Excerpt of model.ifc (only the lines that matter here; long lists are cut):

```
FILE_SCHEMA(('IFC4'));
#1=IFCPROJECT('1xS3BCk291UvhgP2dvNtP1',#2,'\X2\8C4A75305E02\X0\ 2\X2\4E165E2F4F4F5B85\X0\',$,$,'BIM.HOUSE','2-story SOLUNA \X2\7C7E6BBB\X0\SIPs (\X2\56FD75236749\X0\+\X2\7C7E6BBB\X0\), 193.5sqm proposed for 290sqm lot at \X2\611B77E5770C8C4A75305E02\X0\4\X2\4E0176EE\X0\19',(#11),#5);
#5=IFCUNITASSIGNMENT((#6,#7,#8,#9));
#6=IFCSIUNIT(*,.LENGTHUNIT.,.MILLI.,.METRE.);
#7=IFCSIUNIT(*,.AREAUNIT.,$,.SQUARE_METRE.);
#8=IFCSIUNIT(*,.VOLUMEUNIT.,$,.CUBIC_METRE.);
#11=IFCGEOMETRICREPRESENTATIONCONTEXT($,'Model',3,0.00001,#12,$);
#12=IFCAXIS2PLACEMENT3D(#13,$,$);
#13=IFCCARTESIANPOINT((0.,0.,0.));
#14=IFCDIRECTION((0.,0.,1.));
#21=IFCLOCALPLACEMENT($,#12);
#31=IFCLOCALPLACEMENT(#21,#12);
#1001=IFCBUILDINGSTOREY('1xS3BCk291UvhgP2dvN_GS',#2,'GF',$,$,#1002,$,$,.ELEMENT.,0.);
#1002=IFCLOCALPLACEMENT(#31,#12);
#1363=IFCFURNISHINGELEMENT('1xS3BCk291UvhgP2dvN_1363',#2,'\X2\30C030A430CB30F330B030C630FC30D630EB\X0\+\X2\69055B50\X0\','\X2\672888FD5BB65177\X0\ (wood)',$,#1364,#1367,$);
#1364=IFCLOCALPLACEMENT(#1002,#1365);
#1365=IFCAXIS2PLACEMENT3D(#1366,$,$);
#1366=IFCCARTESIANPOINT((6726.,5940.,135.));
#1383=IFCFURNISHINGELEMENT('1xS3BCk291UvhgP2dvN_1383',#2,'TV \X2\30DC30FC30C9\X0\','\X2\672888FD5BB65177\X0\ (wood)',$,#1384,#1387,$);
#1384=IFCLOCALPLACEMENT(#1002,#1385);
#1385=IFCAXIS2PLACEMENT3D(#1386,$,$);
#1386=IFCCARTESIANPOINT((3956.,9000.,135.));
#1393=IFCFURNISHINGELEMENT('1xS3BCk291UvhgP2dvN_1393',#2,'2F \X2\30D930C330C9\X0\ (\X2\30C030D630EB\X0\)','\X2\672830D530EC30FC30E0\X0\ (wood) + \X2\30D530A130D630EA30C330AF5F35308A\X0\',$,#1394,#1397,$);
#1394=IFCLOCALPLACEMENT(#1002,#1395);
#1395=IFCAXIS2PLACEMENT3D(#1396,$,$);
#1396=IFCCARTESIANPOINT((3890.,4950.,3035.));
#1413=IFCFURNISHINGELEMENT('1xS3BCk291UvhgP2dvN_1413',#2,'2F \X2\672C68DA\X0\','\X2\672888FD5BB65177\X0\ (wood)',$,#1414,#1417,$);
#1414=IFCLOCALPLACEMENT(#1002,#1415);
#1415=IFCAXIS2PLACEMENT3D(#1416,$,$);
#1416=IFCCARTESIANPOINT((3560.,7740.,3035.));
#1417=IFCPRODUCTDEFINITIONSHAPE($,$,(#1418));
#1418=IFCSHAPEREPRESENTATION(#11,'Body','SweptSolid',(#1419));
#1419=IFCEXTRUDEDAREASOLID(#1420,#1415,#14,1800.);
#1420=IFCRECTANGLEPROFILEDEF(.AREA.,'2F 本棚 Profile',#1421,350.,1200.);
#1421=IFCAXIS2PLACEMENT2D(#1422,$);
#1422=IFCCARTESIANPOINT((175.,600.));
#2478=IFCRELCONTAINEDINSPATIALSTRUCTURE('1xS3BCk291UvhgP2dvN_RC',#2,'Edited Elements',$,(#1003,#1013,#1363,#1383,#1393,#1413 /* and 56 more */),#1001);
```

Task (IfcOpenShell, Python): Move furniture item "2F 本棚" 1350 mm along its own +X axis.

```python
import ifcopenshell
import ifcopenshell.api.geometry
import ifcopenshell.util.placement
import ifcopenshell.util.unit

model = ifcopenshell.open("model.ifc")
unit_scale = ifcopenshell.util.unit.calculate_unit_scale(model)

item = model.by_id(1413)
matrix = ifcopenshell.util.placement.get_local_placement(item.ObjectPlacement)
matrix[:3, 3] += matrix[:3, 0] * 1.35 / unit_scale
ifcopenshell.api.geometry.edit_object_placement(model, product=item, matrix=matrix, is_si=False)

print(ifcopenshell.util.placement.get_local_placement(item.ObjectPlacement).round(3) + 0.0)

model.write("model_edited.ifc")
```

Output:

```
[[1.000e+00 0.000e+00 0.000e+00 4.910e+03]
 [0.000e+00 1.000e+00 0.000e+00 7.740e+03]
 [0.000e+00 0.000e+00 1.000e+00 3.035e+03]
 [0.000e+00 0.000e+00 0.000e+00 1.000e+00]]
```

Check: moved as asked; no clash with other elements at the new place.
